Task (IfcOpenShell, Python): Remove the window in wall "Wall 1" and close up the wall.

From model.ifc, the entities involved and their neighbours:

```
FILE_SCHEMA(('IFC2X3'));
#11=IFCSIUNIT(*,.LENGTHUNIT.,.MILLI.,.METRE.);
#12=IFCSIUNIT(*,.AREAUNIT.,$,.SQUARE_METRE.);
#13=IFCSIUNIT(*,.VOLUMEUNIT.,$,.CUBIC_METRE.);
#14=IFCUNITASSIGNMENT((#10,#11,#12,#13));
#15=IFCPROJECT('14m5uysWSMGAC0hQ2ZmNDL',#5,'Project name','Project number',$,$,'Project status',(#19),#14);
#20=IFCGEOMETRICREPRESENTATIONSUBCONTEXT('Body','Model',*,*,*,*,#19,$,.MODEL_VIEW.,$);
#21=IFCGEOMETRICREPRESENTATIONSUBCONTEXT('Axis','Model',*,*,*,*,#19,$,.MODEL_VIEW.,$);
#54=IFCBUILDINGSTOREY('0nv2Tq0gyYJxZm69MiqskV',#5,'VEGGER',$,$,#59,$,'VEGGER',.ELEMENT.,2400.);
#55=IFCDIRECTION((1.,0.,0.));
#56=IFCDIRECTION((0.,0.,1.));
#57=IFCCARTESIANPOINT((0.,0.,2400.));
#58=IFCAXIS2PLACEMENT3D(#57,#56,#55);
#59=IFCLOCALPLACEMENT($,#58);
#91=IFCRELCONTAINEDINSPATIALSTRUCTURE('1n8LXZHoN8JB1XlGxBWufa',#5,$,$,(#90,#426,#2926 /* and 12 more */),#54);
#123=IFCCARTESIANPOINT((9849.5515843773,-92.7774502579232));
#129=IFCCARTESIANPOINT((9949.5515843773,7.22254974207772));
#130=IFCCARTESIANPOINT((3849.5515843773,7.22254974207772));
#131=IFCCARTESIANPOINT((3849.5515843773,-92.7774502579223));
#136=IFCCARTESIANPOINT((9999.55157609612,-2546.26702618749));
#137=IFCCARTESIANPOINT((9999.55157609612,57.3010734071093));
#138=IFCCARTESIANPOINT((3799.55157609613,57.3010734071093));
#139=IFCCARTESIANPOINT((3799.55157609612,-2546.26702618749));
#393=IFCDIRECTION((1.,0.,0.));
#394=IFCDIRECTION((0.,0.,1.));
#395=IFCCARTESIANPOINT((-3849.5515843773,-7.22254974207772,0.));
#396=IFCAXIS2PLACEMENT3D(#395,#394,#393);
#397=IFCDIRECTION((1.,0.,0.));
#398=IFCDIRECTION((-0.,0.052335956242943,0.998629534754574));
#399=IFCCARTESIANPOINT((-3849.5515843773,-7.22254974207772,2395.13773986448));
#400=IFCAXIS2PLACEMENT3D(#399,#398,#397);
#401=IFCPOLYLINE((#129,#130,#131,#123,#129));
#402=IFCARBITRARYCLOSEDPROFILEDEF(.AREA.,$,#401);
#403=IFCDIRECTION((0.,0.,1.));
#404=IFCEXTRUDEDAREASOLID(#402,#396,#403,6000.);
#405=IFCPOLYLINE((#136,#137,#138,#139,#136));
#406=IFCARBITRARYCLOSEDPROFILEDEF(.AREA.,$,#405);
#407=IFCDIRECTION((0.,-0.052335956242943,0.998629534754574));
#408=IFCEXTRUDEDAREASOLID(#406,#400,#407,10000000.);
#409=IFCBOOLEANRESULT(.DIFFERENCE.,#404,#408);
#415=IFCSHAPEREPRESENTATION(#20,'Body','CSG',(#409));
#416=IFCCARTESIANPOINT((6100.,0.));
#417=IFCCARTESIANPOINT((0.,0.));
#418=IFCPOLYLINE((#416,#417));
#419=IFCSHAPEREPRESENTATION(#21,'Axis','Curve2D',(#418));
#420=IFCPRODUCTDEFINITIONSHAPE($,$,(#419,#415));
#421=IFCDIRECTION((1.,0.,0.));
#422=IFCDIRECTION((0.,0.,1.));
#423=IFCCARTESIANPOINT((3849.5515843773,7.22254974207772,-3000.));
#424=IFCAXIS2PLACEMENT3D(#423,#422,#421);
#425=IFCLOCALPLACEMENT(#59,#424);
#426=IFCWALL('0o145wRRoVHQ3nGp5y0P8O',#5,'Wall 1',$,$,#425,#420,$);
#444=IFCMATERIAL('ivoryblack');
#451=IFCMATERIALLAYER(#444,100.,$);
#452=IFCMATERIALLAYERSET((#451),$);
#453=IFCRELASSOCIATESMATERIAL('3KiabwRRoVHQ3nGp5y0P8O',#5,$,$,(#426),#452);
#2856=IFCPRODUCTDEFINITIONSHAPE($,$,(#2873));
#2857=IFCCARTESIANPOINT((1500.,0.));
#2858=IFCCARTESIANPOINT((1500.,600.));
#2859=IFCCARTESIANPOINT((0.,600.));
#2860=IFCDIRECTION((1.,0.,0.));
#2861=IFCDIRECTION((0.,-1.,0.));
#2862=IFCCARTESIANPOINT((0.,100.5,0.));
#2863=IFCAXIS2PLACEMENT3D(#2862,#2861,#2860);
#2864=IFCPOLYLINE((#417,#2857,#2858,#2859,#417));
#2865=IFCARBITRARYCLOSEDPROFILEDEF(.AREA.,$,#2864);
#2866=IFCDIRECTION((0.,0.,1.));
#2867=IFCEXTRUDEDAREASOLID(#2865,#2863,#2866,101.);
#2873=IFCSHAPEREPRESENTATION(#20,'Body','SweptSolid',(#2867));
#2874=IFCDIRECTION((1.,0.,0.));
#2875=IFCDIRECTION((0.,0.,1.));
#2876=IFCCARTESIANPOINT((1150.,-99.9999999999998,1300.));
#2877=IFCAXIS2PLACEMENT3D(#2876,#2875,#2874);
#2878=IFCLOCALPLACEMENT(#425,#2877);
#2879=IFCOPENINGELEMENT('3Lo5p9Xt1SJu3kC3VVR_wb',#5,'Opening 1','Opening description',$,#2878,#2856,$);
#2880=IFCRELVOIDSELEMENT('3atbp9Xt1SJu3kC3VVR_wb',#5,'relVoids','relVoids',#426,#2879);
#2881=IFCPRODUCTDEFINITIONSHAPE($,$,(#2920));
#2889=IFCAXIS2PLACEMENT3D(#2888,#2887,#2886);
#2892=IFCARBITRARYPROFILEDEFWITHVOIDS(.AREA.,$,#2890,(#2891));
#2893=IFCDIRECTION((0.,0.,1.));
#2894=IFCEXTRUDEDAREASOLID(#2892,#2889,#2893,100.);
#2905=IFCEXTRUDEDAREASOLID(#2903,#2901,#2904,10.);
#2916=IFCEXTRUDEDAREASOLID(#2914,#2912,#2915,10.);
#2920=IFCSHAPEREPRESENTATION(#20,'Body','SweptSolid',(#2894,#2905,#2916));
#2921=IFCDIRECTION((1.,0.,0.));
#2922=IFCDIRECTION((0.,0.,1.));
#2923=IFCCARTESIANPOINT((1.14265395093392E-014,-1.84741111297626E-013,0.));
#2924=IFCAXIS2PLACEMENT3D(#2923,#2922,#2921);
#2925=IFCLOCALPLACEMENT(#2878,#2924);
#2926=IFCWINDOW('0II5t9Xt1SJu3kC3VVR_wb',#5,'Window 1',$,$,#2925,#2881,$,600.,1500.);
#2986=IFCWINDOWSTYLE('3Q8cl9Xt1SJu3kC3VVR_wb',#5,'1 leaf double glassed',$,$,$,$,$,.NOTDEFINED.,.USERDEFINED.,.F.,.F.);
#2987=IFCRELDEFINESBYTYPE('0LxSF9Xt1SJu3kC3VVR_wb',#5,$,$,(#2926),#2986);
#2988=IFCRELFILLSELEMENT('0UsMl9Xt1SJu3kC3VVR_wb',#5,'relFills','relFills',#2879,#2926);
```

```python
import ifcopenshell
import ifcopenshell.api.feature
import ifcopenshell.api.root
import ifcopenshell.geom
import ifcopenshell.util.shape

model = ifcopenshell.open("model.ifc")
settings = ifcopenshell.geom.settings()


def volume(element):
    """Net volume in cubic metres, openings subtracted."""
    shape = ifcopenshell.geom.create_shape(settings, element)
    return ifcopenshell.util.shape.get_volume(shape.geometry)


window = model.by_guid("0II5t9Xt1SJu3kC3VVR_wb")
opening = window.FillsVoids[0].RelatingOpeningElement
wall = opening.VoidsElements[0].RelatingBuildingElement
before = volume(wall)

ifcopenshell.api.root.remove_product(model, product=window)
ifcopenshell.api.feature.remove_feature(model, feature=opening)

after = volume(wall)

print(f"wall volume {before:.3f} -> {after:.3f} m3")

model.write("model_v2.ifc")
```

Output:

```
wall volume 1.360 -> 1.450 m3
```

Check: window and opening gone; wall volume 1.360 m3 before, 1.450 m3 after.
